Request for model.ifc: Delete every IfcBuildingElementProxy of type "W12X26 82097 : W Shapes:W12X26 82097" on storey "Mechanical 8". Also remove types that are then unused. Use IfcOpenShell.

First a look at what the model holds.

```python
import ifcopenshell
import ifcopenshell.util.element

model = ifcopenshell.open("model.ifc")
print(model.schema)
storey = next(s for s in model.by_type("IfcBuildingStorey") if s.Name == "Mechanical 8")
proxies = [e for e in ifcopenshell.util.element.get_decomposition(storey) if e.is_a("IfcBuildingElementProxy")]
seen = {}
for e in proxies:
    element_type = ifcopenshell.util.element.get_type(e)
    name = element_type.Name if element_type not in (None, e) else None
    seen[name] = seen.get(name, 0) + 1
for name, count in sorted(seen.items(), key=str):
    print(count, "x", name)
```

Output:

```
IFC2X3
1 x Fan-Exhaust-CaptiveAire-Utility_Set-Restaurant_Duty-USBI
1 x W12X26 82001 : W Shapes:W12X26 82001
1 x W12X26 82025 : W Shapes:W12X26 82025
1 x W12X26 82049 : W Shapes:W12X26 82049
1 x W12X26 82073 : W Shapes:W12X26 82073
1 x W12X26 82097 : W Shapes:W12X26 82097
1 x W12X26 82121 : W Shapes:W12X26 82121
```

```python
import ifcopenshell
import ifcopenshell.api.root
import ifcopenshell.util.element

model = ifcopenshell.open("model.ifc")

storey = next(s for s in model.by_type("IfcBuildingStorey") if s.Name == "Mechanical 8")
proxies = [e for e in ifcopenshell.util.element.get_decomposition(storey) if e.is_a("IfcBuildingElementProxy")]
targets = [e for e in proxies if (t := ifcopenshell.util.element.get_type(e)) not in (None, e) and t.Name == "W12X26 82097 : W Shapes:W12X26 82097"]
types = {ifcopenshell.util.element.get_type(e) for e in targets} - {None, *targets}

for e in targets:
    ifcopenshell.api.root.remove_product(model, product=e)
print(len(targets), "removed")

unused = [t for t in types if not ifcopenshell.util.element.get_types(t)]
for t in unused:
    ifcopenshell.api.root.remove_product(model, product=t)
print(len(unused), "unused types removed")

model.write("model_v2.ifc")
```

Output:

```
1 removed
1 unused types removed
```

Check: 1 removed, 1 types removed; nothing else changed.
